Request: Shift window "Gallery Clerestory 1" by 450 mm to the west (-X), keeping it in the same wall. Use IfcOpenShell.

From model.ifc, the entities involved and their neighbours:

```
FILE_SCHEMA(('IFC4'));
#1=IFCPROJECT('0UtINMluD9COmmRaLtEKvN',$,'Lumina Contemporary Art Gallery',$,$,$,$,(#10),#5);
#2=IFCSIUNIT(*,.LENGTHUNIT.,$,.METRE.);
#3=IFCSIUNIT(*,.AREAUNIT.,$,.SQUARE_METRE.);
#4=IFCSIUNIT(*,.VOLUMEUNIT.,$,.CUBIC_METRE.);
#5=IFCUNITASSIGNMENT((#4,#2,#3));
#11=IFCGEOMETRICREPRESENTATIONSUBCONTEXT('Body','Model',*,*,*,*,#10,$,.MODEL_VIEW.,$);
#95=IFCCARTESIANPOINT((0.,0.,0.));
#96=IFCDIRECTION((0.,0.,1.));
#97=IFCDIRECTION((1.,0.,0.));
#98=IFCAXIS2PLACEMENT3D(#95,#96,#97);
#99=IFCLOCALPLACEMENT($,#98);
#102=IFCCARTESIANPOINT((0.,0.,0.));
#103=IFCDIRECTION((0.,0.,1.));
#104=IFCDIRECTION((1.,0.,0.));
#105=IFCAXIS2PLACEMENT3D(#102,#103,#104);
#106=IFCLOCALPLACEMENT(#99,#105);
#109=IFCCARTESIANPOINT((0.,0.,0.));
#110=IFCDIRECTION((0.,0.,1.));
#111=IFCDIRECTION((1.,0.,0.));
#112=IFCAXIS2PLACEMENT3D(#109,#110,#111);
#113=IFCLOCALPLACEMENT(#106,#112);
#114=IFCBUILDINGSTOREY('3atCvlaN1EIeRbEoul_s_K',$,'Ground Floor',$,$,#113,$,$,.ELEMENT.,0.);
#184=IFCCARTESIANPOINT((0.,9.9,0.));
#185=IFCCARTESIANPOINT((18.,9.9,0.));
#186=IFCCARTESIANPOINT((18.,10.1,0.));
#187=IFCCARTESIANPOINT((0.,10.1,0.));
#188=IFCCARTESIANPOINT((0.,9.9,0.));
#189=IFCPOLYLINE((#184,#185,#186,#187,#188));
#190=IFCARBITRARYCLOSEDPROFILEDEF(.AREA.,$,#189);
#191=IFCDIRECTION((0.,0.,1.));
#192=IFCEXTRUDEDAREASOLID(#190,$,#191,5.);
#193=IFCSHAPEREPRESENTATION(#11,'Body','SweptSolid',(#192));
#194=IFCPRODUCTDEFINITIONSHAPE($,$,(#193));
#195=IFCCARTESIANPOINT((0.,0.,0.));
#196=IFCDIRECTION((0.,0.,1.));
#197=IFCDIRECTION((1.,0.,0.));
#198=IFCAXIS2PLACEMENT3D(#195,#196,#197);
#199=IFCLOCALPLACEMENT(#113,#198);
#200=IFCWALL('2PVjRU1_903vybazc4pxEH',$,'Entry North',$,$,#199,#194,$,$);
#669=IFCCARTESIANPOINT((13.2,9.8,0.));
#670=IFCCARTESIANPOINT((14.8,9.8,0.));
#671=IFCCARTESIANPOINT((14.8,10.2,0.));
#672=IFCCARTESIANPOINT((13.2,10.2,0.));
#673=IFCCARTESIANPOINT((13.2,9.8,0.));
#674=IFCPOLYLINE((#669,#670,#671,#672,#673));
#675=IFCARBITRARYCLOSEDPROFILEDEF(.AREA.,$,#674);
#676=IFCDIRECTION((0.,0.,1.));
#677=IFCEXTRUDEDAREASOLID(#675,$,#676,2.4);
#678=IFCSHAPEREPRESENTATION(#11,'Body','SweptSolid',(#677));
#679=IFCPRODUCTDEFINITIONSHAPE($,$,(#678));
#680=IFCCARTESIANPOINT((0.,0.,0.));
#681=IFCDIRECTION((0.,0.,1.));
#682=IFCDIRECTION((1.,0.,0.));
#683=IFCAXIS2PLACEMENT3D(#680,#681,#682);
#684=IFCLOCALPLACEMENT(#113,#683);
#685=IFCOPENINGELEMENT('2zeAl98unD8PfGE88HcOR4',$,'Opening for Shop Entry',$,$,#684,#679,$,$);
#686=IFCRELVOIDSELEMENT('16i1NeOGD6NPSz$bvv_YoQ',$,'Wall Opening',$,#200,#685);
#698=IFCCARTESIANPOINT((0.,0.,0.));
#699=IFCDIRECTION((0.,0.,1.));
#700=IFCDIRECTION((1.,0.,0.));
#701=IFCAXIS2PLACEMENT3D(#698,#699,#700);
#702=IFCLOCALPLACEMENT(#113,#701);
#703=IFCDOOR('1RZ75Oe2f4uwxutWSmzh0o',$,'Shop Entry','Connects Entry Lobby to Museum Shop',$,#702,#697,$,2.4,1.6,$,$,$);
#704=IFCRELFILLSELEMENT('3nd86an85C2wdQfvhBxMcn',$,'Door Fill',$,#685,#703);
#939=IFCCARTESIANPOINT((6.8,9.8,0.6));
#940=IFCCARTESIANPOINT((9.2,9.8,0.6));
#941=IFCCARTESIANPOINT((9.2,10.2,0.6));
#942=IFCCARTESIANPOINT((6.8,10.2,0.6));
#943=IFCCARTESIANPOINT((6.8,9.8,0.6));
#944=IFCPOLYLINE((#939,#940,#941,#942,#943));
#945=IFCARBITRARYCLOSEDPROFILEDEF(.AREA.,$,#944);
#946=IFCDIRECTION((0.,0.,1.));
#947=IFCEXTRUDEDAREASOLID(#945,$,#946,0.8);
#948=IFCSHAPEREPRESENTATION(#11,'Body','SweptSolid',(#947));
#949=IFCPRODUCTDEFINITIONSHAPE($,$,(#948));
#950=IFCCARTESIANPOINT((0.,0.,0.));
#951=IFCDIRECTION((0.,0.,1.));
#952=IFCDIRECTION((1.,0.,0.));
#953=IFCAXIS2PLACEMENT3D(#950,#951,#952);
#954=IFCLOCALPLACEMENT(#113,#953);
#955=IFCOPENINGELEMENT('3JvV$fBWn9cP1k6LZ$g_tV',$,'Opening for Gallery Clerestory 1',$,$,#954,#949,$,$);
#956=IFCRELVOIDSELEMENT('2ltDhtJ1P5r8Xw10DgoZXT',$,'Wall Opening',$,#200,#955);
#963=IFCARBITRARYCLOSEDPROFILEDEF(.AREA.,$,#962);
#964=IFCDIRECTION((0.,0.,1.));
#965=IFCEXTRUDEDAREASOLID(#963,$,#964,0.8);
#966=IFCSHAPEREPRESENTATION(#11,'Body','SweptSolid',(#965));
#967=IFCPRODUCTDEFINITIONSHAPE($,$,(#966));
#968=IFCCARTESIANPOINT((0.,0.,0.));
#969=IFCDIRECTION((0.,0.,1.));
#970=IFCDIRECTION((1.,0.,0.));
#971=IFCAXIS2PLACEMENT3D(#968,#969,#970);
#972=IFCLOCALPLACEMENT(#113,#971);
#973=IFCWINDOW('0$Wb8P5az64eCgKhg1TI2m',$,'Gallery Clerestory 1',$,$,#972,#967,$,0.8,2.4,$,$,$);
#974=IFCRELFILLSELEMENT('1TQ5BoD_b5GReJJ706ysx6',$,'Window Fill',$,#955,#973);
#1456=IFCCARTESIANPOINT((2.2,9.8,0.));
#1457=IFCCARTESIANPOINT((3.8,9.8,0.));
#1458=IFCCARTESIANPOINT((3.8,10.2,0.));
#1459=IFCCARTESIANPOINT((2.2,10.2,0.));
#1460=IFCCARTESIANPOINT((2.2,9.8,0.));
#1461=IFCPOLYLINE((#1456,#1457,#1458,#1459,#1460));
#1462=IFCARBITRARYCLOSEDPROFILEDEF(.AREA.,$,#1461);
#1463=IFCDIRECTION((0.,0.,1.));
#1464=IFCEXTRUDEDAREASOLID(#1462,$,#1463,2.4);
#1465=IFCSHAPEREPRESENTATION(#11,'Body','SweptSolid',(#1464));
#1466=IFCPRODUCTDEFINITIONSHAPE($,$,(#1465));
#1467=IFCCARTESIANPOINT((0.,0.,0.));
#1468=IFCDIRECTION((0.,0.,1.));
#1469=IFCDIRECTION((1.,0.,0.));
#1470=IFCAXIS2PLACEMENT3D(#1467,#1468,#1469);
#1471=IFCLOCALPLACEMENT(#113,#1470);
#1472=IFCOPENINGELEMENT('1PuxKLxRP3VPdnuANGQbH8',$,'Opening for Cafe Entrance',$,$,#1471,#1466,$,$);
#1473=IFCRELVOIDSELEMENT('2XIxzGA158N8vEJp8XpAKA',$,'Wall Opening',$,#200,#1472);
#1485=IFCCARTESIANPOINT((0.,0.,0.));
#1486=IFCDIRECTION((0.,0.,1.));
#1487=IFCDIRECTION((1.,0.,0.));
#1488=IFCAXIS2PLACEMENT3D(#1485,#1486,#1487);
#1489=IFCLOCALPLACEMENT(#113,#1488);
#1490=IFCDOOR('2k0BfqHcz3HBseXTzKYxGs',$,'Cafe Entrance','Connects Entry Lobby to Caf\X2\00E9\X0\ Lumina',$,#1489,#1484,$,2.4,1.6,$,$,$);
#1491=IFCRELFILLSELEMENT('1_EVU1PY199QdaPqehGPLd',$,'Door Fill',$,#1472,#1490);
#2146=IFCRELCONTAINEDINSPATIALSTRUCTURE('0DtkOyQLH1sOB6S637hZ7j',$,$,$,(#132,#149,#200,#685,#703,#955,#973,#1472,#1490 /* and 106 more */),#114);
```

```python
import ifcopenshell
import ifcopenshell.api.geometry
import ifcopenshell.util.placement
import ifcopenshell.util.unit

model = ifcopenshell.open("model.ifc")
unit_scale = ifcopenshell.util.unit.calculate_unit_scale(model)

window = model.by_guid("0$Wb8P5az64eCgKhg1TI2m")
opening = window.FillsVoids[0].RelatingOpeningElement
wall = opening.VoidsElements[0].RelatingBuildingElement

wall_matrix = ifcopenshell.util.placement.get_local_placement(wall.ObjectPlacement)
shift = wall_matrix[:3, 0] * -0.45 / unit_scale
before = ifcopenshell.util.placement.get_local_placement(window.ObjectPlacement)[:3, 3].copy()

# The window is not placed relative to its opening, so move both.
for product in (opening, window):
    matrix = ifcopenshell.util.placement.get_local_placement(product.ObjectPlacement)
    matrix[:3, 3] += shift
    ifcopenshell.api.geometry.edit_object_placement(model, product=product, matrix=matrix, is_si=False)

after = ifcopenshell.util.placement.get_local_placement(window.ObjectPlacement)[:3, 3]
print("window moved by", (after - before).round(3) + 0.0)

model.write("model_v2.ifc")
```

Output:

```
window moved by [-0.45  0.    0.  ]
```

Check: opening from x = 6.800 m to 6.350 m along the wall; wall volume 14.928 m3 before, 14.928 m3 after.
